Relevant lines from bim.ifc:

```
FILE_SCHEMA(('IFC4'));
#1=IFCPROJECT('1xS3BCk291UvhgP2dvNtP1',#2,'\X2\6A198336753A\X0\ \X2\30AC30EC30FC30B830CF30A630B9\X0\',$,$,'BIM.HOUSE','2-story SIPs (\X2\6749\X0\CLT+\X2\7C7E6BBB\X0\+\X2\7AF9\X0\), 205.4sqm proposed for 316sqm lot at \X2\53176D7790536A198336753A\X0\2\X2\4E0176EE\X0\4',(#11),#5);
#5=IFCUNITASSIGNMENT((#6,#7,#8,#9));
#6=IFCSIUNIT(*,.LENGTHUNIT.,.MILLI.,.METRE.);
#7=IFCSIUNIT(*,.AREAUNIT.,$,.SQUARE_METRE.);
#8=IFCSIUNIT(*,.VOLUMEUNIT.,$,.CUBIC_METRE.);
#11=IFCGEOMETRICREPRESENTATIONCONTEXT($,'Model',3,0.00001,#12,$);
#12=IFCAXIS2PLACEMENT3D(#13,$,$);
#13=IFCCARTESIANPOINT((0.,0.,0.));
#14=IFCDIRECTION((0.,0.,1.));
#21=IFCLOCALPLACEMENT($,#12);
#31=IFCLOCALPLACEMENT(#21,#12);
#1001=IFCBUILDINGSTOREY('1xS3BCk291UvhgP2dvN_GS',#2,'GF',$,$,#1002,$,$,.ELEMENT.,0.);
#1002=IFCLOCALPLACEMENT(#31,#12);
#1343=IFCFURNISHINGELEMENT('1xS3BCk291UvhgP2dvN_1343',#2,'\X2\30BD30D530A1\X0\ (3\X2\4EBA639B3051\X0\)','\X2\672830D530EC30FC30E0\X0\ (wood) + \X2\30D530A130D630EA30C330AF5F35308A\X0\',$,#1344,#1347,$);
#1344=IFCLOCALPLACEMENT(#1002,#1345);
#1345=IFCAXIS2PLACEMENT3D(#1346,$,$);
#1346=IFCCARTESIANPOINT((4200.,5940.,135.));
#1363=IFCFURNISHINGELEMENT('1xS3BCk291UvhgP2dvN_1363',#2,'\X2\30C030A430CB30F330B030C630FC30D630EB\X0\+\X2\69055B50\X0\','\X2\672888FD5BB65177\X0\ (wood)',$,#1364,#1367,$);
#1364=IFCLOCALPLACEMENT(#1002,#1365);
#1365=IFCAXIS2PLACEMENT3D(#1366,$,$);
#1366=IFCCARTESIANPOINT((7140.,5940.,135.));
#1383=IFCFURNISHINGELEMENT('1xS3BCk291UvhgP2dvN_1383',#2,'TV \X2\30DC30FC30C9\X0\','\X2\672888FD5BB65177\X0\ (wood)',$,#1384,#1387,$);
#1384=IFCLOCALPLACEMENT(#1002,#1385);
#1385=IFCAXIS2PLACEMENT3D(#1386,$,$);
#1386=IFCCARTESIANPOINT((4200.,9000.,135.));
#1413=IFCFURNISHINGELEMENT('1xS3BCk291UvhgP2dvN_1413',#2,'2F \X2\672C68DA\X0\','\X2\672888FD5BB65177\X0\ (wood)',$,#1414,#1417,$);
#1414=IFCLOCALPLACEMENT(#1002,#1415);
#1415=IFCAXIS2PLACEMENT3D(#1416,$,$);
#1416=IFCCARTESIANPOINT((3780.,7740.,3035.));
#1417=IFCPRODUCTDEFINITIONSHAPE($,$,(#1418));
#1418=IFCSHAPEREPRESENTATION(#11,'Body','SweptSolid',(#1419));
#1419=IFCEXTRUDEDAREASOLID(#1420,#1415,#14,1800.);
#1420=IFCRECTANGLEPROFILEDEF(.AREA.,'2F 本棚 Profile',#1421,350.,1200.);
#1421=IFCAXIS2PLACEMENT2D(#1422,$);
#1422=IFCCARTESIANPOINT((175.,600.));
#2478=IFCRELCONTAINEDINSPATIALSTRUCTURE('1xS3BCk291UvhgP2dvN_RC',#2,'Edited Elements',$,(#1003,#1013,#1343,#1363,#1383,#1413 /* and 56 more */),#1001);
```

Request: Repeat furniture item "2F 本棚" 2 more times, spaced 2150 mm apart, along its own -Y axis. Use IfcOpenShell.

```python
import ifcopenshell
import ifcopenshell.api.geometry
import ifcopenshell.api.root
import ifcopenshell.util.element
import ifcopenshell.util.placement
import ifcopenshell.util.unit

model = ifcopenshell.open("bim.ifc")
unit_scale = ifcopenshell.util.unit.calculate_unit_scale(model)


def reuse_history(source, copy):
    """copy_class also copies each property set's owner history, people and application; keep the originals."""
    for rel in copy.IsDefinedBy:
        if rel.is_a("IfcRelDefinesByProperties") and (history := rel.RelatingPropertyDefinition.OwnerHistory):
            rel.RelatingPropertyDefinition.OwnerHistory = source.OwnerHistory
            ifcopenshell.util.element.remove_deep2(model, history)


source = model.by_id(1413)
base = ifcopenshell.util.placement.get_local_placement(source.ObjectPlacement)
step = -base[:3, 1] * 2.15 / unit_scale

for i in range(1, 3):
    copy = ifcopenshell.api.root.copy_class(model, product=source)
    copy.Representation = ifcopenshell.util.element.copy_deep(
        model, source.Representation, exclude=["IfcGeometricRepresentationContext", "IfcRepresentationMap"]
    )
    reuse_history(source, copy)
    matrix = base.copy()
    matrix[:3, 3] += i * step
    print("added at", matrix[:3, 3].round(3) + 0.0)
    ifcopenshell.api.geometry.edit_object_placement(model, product=copy, matrix=matrix, is_si=False)

model.write("bim_updated.ifc")
```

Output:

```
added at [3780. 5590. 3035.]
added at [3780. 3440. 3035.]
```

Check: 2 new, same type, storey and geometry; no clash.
